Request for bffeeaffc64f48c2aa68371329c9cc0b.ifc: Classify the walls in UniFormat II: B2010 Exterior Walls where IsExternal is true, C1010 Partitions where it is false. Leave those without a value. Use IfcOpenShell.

First a look at what the model holds.

```python
import ifcopenshell
import ifcopenshell.util.element

model = ifcopenshell.open("bffeeaffc64f48c2aa68371329c9cc0b.ifc")
print(model.schema)
print("classifications:", [c.Name for c in model.by_type("IfcClassification")])
values = [ifcopenshell.util.element.get_pset(e, "Pset_WallCommon", "IsExternal") for e in model.by_type("IfcWall")]
for value in (True, False, None):
    print("IsExternal", value, values.count(value))
```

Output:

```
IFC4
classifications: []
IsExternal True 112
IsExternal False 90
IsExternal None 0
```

```python
import ifcopenshell
import ifcopenshell.api.classification
import ifcopenshell.util.element

model = ifcopenshell.open("bffeeaffc64f48c2aa68371329c9cc0b.ifc")

system = ifcopenshell.api.classification.add_classification(model, classification="UniFormat II")

walls = model.by_type("IfcWall")
external = {e: ifcopenshell.util.element.get_pset(e, "Pset_WallCommon", "IsExternal") for e in walls}
for flag, code, name in ((True, "B2010", "Exterior Walls"), (False, "C1010", "Partitions")):
    products = [e for e in walls if external[e] is flag]
    ifcopenshell.api.classification.add_reference(
        model, products=products, classification=system, identification=code, name=name
    )
    print(code, len(products))

model.write("bffeeaffc64f48c2aa68371329c9cc0b_updated.ifc")
```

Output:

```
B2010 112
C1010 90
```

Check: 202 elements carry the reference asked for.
